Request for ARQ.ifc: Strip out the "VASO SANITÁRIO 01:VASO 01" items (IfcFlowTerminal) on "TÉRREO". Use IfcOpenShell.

First a look at what the model holds.

```python
import ifcopenshell
import ifcopenshell.util.element

model = ifcopenshell.open("ARQ.ifc")
print(model.schema)
storey = next(s for s in model.by_type("IfcBuildingStorey") if s.Name == "TÉRREO")
terminals = [e for e in ifcopenshell.util.element.get_decomposition(storey) if e.is_a("IfcFlowTerminal")]
seen = {}
for e in terminals:
    element_type = ifcopenshell.util.element.get_type(e)
    name = element_type.Name if element_type not in (None, e) else None
    seen[name] = seen.get(name, 0) + 1
for name, count in sorted(seen.items(), key=str):
    print(count, "x", name)
```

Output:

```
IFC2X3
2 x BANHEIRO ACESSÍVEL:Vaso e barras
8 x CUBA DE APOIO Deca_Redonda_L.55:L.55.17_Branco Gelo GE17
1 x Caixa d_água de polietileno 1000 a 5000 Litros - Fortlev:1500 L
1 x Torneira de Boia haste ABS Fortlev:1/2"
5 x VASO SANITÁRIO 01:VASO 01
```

```python
import ifcopenshell
import ifcopenshell.api.root
import ifcopenshell.util.element

model = ifcopenshell.open("ARQ.ifc")

storey = next(s for s in model.by_type("IfcBuildingStorey") if s.Name == "TÉRREO")
terminals = [e for e in ifcopenshell.util.element.get_decomposition(storey) if e.is_a("IfcFlowTerminal")]
targets = [e for e in terminals if (t := ifcopenshell.util.element.get_type(e)) not in (None, e) and t.Name == "VASO SANITÁRIO 01:VASO 01"]

for e in targets:
    ifcopenshell.api.root.remove_product(model, product=e)
print(len(targets), "removed")

model.write("ARQ_edited.ifc")
```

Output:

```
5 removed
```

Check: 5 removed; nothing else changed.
